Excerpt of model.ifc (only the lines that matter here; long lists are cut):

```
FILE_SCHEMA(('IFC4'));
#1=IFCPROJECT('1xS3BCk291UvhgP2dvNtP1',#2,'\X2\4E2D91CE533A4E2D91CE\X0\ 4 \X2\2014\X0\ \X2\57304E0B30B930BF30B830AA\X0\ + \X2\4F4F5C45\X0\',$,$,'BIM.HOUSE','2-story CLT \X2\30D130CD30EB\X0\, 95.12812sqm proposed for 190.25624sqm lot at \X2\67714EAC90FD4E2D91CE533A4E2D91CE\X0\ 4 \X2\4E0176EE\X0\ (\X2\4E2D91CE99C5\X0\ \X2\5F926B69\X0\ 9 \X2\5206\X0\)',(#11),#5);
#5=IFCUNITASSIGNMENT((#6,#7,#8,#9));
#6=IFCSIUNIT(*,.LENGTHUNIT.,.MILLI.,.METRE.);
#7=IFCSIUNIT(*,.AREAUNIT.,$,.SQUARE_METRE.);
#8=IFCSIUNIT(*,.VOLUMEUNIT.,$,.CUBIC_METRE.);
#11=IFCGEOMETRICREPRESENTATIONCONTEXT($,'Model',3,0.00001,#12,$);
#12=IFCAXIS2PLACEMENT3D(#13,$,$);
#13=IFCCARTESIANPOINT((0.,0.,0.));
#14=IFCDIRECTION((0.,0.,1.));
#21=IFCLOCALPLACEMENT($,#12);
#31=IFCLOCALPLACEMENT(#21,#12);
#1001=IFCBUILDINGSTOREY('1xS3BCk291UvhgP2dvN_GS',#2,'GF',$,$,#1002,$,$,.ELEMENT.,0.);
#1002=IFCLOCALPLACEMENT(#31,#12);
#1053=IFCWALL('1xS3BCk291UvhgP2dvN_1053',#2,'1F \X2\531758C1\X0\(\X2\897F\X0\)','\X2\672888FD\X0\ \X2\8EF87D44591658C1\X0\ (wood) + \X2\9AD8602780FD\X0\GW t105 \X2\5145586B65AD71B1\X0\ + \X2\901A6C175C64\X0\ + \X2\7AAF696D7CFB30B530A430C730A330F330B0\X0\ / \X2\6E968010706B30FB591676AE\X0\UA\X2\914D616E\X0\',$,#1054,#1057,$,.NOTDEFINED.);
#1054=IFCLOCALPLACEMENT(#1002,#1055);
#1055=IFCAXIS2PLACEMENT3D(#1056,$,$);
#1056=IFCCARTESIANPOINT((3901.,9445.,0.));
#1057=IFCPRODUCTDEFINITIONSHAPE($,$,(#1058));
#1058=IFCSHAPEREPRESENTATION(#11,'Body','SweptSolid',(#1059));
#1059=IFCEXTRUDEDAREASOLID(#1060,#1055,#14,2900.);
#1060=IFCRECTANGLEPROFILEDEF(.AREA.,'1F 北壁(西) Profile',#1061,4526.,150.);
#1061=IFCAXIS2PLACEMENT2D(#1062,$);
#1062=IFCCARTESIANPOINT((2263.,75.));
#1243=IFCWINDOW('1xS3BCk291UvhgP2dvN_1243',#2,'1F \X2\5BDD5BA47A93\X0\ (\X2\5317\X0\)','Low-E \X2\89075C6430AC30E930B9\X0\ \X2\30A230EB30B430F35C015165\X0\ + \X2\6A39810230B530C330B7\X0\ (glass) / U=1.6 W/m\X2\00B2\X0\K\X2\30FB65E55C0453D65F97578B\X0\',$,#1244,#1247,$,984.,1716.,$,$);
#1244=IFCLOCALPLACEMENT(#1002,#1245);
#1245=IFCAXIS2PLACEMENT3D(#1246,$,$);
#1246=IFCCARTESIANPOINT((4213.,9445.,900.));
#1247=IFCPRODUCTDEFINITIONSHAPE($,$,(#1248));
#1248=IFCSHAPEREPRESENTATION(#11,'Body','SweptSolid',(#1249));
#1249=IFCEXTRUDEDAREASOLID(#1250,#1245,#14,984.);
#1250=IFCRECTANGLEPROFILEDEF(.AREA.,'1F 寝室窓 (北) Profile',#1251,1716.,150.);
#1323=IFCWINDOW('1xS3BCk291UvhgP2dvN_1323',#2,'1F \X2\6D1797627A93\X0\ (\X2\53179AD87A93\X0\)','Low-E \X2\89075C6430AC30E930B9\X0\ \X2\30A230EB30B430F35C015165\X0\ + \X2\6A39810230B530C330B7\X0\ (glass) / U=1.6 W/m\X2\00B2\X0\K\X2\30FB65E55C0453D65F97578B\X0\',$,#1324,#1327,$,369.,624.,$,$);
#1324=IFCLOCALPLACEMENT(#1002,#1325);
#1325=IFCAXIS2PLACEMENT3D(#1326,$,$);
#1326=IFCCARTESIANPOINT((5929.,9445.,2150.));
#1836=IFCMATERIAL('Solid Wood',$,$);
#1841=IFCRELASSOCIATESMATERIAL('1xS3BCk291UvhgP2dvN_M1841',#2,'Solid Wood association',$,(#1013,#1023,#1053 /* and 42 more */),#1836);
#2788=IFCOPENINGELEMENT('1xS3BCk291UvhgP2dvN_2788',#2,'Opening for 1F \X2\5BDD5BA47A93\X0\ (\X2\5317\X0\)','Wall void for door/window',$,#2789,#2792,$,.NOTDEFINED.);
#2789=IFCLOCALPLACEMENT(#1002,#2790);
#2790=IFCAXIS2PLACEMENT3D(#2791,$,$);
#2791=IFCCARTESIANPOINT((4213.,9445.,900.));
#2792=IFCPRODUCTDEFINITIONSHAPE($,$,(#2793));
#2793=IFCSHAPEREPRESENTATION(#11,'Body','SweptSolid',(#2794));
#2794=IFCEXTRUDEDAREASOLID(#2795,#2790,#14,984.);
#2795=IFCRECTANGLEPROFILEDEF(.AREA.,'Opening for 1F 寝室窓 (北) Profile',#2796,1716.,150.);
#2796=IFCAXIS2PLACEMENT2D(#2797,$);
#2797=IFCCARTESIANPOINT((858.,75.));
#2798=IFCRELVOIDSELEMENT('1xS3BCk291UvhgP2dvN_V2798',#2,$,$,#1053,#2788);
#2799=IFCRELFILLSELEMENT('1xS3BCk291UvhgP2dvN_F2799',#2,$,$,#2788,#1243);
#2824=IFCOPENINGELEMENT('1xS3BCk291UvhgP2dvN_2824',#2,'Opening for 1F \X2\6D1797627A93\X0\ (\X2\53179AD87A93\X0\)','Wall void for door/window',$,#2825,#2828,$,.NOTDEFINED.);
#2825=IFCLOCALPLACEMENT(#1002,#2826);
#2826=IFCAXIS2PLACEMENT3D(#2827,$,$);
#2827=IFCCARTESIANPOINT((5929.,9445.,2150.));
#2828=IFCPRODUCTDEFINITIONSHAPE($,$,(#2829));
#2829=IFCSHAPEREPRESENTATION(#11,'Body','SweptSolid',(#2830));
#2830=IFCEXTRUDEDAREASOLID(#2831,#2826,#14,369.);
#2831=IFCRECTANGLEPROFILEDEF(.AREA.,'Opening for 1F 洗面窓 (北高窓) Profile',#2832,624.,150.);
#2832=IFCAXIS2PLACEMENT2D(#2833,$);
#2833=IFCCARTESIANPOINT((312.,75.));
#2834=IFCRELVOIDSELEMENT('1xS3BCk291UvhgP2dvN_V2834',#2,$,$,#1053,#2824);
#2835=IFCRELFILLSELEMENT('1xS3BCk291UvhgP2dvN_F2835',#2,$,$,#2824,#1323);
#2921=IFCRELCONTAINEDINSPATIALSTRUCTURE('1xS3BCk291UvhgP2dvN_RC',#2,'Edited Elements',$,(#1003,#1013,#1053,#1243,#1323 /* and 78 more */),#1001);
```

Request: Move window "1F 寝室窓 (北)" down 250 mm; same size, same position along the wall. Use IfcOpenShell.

```python
import numpy as np
import ifcopenshell
import ifcopenshell.api.geometry
import ifcopenshell.util.placement
import ifcopenshell.util.unit

model = ifcopenshell.open("model.ifc")
unit_scale = ifcopenshell.util.unit.calculate_unit_scale(model)

window = model.by_guid("1xS3BCk291UvhgP2dvN_1243")
opening = window.FillsVoids[0].RelatingOpeningElement
dz = -0.25 / unit_scale

shift = np.array([0.0, 0.0, dz])
# The window is not placed relative to its opening, so move both.
for product in (opening, window):
    matrix = ifcopenshell.util.placement.get_local_placement(product.ObjectPlacement)
    matrix[:3, 3] += shift
    ifcopenshell.api.geometry.edit_object_placement(model, product=product, matrix=matrix, is_si=False)

print(f"moved by {dz * unit_scale:+.3f} m")

model.write("model_v2.ifc")
```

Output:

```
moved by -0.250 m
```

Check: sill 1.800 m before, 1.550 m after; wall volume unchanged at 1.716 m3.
